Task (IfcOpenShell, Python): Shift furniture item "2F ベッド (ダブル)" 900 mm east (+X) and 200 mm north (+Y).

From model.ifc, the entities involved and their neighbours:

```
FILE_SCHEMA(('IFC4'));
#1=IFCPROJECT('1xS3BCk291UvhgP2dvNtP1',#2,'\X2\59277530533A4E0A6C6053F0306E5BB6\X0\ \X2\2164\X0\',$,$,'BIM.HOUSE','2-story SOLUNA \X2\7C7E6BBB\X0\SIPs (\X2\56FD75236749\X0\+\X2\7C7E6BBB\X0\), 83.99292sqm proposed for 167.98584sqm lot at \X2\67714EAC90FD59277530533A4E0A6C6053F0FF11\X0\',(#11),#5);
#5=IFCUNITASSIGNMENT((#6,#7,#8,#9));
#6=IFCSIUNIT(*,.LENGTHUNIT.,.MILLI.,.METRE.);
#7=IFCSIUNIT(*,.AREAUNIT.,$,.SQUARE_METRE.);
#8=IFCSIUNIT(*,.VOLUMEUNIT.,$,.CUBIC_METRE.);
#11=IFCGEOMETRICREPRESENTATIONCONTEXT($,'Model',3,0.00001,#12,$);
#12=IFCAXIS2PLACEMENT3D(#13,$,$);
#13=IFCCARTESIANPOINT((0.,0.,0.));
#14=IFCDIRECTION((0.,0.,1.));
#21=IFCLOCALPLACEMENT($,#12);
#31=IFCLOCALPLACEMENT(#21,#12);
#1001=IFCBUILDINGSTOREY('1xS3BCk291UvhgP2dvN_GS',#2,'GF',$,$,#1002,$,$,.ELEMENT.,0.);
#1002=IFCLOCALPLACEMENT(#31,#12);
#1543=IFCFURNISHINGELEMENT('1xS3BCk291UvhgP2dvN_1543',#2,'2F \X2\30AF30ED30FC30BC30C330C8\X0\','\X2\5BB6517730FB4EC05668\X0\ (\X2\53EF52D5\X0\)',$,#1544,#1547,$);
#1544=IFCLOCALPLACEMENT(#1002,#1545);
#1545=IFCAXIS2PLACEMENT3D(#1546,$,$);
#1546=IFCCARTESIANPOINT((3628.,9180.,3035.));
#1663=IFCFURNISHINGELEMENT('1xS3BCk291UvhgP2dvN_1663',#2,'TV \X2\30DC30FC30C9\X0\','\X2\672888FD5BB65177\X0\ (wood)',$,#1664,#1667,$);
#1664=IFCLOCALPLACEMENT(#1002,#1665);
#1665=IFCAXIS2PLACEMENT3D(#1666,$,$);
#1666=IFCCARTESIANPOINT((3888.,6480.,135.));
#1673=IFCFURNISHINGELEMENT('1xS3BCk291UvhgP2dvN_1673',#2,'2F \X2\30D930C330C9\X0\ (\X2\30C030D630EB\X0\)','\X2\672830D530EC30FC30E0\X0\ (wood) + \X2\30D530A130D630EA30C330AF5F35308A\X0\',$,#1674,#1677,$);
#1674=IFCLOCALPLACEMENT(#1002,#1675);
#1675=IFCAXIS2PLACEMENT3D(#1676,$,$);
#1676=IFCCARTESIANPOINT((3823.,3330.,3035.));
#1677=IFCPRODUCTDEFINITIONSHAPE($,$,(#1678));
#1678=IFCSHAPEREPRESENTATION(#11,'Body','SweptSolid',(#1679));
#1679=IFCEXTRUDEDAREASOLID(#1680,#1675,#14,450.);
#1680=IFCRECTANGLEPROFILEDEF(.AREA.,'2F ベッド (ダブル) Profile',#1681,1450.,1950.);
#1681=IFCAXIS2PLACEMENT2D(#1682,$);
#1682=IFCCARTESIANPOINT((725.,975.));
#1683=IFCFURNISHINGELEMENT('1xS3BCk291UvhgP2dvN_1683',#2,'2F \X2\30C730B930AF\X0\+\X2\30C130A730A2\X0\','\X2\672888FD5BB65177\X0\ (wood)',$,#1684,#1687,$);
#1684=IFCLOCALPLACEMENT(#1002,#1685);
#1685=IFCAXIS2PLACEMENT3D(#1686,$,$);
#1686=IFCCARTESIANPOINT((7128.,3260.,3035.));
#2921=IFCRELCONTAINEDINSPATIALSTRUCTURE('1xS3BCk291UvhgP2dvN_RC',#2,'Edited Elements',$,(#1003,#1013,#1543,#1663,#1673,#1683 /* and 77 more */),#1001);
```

```python
import ifcopenshell
import ifcopenshell.api.geometry
import ifcopenshell.util.placement
import ifcopenshell.util.unit

model = ifcopenshell.open("model.ifc")
unit_scale = ifcopenshell.util.unit.calculate_unit_scale(model)

item = model.by_id(1673)
matrix = ifcopenshell.util.placement.get_local_placement(item.ObjectPlacement)
matrix[0, 3] += 0.9 / unit_scale
matrix[1, 3] += 0.2 / unit_scale
ifcopenshell.api.geometry.edit_object_placement(model, product=item, matrix=matrix, is_si=False)

print(ifcopenshell.util.placement.get_local_placement(item.ObjectPlacement).round(3) + 0.0)

model.write("model_rev.ifc")
```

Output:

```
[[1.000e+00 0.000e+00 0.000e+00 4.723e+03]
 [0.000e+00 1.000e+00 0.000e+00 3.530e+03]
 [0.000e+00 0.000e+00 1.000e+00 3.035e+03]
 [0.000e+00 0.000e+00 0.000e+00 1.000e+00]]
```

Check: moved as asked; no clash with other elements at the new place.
